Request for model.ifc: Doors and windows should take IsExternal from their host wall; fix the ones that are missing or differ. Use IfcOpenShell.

First a look at what the model holds.

```python
import ifcopenshell
import ifcopenshell.util.element

model = ifcopenshell.open("model.ifc")
print(model.schema)
seen = {}
for e in model.by_type("IfcDoor") + model.by_type("IfcWindow"):
    if not e.FillsVoids:
        continue
    host = e.FillsVoids[0].RelatingOpeningElement.VoidsElements[0].RelatingBuildingElement
    own = ifcopenshell.util.element.get_pset(e, f"Pset_{e.is_a()[3:].removesuffix('StandardCase')}Common", "IsExternal")
    wall = ifcopenshell.util.element.get_pset(host, "Pset_WallCommon", "IsExternal")
    seen[e.is_a(), own, wall] = seen.get((e.is_a(), own, wall), 0) + 1
for (cls, own, wall), count in sorted(seen.items(), key=str):
    print(count, cls, "IsExternal:", own, "| host wall:", wall)
```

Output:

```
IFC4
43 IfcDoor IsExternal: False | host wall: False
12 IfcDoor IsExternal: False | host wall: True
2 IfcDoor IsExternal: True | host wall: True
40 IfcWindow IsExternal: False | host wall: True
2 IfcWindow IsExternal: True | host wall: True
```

```python
import ifcopenshell
import ifcopenshell.api.pset
import ifcopenshell.util.element

model = ifcopenshell.open("model.ifc")

count = 0
for ifc_class, pset_name in (("IfcDoor", "Pset_DoorCommon"), ("IfcWindow", "Pset_WindowCommon")):
    for e in model.by_type(ifc_class):
        if not e.FillsVoids:
            continue
        host = e.FillsVoids[0].RelatingOpeningElement.VoidsElements[0].RelatingBuildingElement
        external = ifcopenshell.util.element.get_pset(host, "Pset_WallCommon", "IsExternal")
        if external is None or ifcopenshell.util.element.get_pset(e, pset_name, "IsExternal") == external:
            continue
        pset = ifcopenshell.api.pset.add_pset(model, product=e, name=pset_name)
        ifcopenshell.api.pset.edit_pset(model, pset=pset, properties={"IsExternal": external})
        count += 1

print(count, "updated")

model.write("model_updated.ifc")
```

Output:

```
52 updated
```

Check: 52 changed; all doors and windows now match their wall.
